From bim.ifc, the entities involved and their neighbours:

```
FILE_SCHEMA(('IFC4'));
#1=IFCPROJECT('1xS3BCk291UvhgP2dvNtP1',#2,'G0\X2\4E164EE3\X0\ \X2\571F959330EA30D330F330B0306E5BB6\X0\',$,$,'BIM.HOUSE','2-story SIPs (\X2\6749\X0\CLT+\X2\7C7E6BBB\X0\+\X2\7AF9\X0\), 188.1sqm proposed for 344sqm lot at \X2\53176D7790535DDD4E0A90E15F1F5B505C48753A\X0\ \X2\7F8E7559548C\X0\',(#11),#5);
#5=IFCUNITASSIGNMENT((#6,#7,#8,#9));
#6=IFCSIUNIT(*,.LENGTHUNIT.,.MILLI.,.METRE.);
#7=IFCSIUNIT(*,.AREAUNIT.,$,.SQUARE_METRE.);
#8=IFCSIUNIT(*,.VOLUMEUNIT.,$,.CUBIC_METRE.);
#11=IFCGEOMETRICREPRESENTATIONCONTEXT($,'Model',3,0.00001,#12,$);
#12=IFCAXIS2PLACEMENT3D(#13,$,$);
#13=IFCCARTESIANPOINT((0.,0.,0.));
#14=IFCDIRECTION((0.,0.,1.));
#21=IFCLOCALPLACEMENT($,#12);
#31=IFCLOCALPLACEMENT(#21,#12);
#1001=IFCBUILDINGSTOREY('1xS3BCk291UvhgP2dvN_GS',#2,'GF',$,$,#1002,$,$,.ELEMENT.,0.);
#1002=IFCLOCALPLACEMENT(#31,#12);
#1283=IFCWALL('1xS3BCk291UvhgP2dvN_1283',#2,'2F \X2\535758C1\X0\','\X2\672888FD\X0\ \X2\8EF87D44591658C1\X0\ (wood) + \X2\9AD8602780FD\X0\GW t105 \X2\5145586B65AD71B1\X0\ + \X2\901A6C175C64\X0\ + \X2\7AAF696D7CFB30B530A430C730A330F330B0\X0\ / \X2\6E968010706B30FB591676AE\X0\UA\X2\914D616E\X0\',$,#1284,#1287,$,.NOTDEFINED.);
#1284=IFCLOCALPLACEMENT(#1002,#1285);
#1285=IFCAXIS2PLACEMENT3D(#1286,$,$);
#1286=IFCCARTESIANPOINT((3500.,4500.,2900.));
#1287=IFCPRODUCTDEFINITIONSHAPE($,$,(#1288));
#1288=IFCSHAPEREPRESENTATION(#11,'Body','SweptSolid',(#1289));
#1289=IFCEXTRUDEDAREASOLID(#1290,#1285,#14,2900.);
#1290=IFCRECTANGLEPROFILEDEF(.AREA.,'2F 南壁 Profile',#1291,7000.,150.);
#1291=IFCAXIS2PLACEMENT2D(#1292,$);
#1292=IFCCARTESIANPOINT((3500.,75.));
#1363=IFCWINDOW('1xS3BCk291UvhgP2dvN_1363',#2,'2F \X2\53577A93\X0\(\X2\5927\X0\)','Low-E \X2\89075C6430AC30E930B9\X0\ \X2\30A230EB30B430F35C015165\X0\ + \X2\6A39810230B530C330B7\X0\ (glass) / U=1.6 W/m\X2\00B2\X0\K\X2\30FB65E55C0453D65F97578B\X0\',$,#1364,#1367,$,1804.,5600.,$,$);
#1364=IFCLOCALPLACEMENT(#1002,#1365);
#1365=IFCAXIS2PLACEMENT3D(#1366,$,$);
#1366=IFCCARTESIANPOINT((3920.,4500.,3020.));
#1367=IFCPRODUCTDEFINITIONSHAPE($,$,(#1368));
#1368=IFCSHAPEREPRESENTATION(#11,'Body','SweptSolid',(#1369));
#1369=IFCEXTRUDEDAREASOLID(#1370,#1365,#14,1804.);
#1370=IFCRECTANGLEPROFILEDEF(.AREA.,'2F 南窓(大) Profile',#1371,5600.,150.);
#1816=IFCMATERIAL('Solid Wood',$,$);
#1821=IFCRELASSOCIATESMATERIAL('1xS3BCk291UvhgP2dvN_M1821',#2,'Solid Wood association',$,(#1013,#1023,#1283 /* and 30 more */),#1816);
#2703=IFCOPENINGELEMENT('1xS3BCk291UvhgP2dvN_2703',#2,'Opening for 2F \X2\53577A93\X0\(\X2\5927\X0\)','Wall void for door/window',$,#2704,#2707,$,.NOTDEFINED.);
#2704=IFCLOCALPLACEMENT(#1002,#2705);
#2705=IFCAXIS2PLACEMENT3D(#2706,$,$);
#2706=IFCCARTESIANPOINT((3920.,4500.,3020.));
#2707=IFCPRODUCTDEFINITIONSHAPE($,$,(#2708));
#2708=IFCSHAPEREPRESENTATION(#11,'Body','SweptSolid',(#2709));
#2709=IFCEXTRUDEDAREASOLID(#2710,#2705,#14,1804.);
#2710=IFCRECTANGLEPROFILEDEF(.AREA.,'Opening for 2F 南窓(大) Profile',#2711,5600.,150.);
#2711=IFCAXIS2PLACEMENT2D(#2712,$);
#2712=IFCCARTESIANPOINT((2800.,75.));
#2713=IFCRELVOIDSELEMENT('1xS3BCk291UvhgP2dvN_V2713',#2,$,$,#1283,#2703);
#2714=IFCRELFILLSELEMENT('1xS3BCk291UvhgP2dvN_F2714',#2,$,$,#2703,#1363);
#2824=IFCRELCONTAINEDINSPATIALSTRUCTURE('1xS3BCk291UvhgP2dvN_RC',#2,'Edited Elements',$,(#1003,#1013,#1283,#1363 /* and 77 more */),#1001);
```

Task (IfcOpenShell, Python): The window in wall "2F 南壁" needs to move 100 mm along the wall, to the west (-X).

```python
import ifcopenshell
import ifcopenshell.api.geometry
import ifcopenshell.util.placement
import ifcopenshell.util.unit

model = ifcopenshell.open("bim.ifc")
unit_scale = ifcopenshell.util.unit.calculate_unit_scale(model)

window = model.by_guid("1xS3BCk291UvhgP2dvN_1363")
opening = window.FillsVoids[0].RelatingOpeningElement
wall = opening.VoidsElements[0].RelatingBuildingElement

wall_matrix = ifcopenshell.util.placement.get_local_placement(wall.ObjectPlacement)
shift = wall_matrix[:3, 0] * -0.1 / unit_scale
before = ifcopenshell.util.placement.get_local_placement(window.ObjectPlacement)[:3, 3].copy()

# The window is not placed relative to its opening, so move both.
for product in (opening, window):
    matrix = ifcopenshell.util.placement.get_local_placement(product.ObjectPlacement)
    matrix[:3, 3] += shift
    ifcopenshell.api.geometry.edit_object_placement(model, product=product, matrix=matrix, is_si=False)

after = ifcopenshell.util.placement.get_local_placement(window.ObjectPlacement)[:3, 3]
print("window moved by", (after - before).round(3) + 0.0)

model.write("bim_rev.ifc")
```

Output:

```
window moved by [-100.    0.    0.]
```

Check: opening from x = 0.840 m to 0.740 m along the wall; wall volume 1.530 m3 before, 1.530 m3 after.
